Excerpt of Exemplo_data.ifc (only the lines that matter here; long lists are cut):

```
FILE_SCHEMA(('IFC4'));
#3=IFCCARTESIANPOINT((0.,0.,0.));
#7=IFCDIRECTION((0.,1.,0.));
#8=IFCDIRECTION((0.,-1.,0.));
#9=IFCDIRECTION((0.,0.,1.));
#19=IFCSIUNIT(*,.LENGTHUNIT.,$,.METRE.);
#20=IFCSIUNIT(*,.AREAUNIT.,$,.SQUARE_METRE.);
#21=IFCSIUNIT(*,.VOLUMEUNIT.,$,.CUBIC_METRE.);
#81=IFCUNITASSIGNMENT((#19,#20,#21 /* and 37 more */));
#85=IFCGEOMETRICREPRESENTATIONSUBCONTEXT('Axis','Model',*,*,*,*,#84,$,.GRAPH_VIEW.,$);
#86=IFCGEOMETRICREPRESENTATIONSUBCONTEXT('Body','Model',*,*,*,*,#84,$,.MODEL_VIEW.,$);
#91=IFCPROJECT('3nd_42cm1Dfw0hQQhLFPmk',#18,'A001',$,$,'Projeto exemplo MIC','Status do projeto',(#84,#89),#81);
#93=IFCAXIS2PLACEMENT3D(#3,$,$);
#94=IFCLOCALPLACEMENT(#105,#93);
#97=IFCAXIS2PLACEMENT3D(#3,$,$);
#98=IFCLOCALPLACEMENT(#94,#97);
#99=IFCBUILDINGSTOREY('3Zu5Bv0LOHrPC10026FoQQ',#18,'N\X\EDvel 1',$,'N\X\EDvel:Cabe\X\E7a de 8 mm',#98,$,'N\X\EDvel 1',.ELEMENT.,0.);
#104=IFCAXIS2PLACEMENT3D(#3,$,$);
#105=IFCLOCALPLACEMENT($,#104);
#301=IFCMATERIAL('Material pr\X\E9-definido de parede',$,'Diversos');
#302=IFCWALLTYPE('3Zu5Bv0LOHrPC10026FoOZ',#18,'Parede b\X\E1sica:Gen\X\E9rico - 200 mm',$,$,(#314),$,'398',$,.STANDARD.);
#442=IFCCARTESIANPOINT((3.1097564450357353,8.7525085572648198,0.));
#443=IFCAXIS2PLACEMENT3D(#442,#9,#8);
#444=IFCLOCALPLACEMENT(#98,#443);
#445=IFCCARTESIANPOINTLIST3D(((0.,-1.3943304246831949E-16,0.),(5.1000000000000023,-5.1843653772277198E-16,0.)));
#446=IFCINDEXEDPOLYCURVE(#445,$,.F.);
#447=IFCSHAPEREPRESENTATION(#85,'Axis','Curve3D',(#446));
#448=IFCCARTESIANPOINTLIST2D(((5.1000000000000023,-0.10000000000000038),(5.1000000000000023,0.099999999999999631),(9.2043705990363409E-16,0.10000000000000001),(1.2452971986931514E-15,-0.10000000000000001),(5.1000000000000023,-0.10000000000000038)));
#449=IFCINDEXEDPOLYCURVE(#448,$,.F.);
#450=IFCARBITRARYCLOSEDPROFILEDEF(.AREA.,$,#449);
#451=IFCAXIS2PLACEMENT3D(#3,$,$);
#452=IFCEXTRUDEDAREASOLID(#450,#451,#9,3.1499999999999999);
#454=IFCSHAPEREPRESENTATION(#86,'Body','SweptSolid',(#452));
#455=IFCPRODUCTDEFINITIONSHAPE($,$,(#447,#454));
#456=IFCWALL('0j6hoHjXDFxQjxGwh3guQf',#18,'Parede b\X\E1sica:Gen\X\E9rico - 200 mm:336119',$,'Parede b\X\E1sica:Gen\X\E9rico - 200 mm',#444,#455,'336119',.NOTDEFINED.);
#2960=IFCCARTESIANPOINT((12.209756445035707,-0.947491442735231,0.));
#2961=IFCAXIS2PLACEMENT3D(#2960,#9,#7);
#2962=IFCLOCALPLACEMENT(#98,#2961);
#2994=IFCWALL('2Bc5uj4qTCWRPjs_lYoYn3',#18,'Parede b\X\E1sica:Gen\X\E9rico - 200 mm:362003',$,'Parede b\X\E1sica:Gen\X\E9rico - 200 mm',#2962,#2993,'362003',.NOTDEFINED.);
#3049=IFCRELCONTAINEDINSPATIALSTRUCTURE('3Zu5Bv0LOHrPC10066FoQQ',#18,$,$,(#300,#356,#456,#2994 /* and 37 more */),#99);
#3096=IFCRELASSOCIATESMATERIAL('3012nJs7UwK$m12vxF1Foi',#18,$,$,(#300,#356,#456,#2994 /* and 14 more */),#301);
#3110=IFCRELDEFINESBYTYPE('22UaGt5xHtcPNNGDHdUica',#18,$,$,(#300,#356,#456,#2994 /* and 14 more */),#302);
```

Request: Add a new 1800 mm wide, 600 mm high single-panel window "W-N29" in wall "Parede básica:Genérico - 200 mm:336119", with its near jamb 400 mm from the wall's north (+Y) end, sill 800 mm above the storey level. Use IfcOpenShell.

```python
import numpy as np
import ifcopenshell
import ifcopenshell.api.feature
import ifcopenshell.api.geometry
import ifcopenshell.api.root
import ifcopenshell.api.spatial
import ifcopenshell.geom
import ifcopenshell.util.element
import ifcopenshell.util.placement
import ifcopenshell.util.representation
import ifcopenshell.util.shape
import ifcopenshell.util.unit

model = ifcopenshell.open("Exemplo_data.ifc")
unit_scale = ifcopenshell.util.unit.calculate_unit_scale(model)
settings = ifcopenshell.geom.settings()


def volume(element):
    """Net volume in cubic metres, openings subtracted."""
    shape = ifcopenshell.geom.create_shape(settings, element)
    return ifcopenshell.util.shape.get_volume(shape.geometry)


wall = model.by_guid("0j6hoHjXDFxQjxGwh3guQf")
storey = ifcopenshell.util.element.get_container(wall, ifc_class="IfcBuildingStorey")
context = ifcopenshell.util.representation.get_context(model, "Model", "Body", "MODEL_VIEW")
before = volume(wall)

width, height, from_end, sill = 1.8, 0.6, 0.4, 0.8  # metres

# The wall runs along its own X axis, and the end named is its -X end.
wall_shape = ifcopenshell.geom.create_shape(settings, wall)
x, y, z = ifcopenshell.util.shape.get_vertices(wall_shape.geometry).T
start = x.min() + from_end
face, thickness = float(y.min()), float(y.max() - y.min())
wall_matrix = ifcopenshell.util.placement.get_local_placement(wall.ObjectPlacement)
level = ifcopenshell.util.placement.get_local_placement(storey.ObjectPlacement)[2, 3]


def in_wall(x, y):
    """Placement at x, y metres in the wall's axes, at sill height."""
    matrix = wall_matrix.copy()
    matrix[:, 3] = wall_matrix @ np.array([x / unit_scale, y / unit_scale, 0.0, 1.0])
    matrix[2, 3] = level + sill / unit_scale
    return matrix


# Opening: a box that overshoots both wall faces by 50 mm.
opening = ifcopenshell.api.root.create_entity(model, ifc_class="IfcOpeningElement", predefined_type="OPENING")
box = ifcopenshell.api.geometry.add_wall_representation(
    model, context=context, length=width, height=height, thickness=thickness + 0.1
)
ifcopenshell.api.geometry.assign_representation(model, product=opening, representation=box)
ifcopenshell.api.geometry.edit_object_placement(model, product=opening, matrix=in_wall(start, face - 0.05), is_si=False)
ifcopenshell.api.feature.add_feature(model, feature=opening, element=wall)

window = ifcopenshell.api.root.create_entity(model, ifc_class="IfcWindow", name="W-N29", predefined_type="WINDOW")
window.OverallWidth, window.OverallHeight = width / unit_scale, height / unit_scale
window.PartitioningType = "SINGLE_PANEL"
body = ifcopenshell.api.geometry.add_window_representation(
    model,
    context=context,
    overall_width=window.OverallWidth,
    overall_height=window.OverallHeight,
    partition_type="SINGLE_PANEL",
)
ifcopenshell.api.geometry.assign_representation(model, product=window, representation=body)
ifcopenshell.api.spatial.assign_container(model, products=[window], relating_structure=storey)
ifcopenshell.api.feature.add_filling(model, opening=opening, element=window)

# Centre the window in the wall's thickness.
ifcopenshell.api.geometry.edit_object_placement(model, product=window, matrix=in_wall(start, face), is_si=False)
window_shape = ifcopenshell.geom.create_shape(settings, window)
depth = ifcopenshell.util.shape.get_vertices(window_shape.geometry)[:, 1]
offset = face + thickness / 2 - (depth.min() + depth.max()) / 2
ifcopenshell.api.geometry.edit_object_placement(model, product=window, matrix=in_wall(start, offset), is_si=False)

after = volume(wall)

print(f"wall volume {before:.3f} -> {after:.3f} m3")

model.write("Exemplo_data_v2.ifc")
```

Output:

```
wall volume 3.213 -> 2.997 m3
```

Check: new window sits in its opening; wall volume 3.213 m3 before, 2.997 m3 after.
